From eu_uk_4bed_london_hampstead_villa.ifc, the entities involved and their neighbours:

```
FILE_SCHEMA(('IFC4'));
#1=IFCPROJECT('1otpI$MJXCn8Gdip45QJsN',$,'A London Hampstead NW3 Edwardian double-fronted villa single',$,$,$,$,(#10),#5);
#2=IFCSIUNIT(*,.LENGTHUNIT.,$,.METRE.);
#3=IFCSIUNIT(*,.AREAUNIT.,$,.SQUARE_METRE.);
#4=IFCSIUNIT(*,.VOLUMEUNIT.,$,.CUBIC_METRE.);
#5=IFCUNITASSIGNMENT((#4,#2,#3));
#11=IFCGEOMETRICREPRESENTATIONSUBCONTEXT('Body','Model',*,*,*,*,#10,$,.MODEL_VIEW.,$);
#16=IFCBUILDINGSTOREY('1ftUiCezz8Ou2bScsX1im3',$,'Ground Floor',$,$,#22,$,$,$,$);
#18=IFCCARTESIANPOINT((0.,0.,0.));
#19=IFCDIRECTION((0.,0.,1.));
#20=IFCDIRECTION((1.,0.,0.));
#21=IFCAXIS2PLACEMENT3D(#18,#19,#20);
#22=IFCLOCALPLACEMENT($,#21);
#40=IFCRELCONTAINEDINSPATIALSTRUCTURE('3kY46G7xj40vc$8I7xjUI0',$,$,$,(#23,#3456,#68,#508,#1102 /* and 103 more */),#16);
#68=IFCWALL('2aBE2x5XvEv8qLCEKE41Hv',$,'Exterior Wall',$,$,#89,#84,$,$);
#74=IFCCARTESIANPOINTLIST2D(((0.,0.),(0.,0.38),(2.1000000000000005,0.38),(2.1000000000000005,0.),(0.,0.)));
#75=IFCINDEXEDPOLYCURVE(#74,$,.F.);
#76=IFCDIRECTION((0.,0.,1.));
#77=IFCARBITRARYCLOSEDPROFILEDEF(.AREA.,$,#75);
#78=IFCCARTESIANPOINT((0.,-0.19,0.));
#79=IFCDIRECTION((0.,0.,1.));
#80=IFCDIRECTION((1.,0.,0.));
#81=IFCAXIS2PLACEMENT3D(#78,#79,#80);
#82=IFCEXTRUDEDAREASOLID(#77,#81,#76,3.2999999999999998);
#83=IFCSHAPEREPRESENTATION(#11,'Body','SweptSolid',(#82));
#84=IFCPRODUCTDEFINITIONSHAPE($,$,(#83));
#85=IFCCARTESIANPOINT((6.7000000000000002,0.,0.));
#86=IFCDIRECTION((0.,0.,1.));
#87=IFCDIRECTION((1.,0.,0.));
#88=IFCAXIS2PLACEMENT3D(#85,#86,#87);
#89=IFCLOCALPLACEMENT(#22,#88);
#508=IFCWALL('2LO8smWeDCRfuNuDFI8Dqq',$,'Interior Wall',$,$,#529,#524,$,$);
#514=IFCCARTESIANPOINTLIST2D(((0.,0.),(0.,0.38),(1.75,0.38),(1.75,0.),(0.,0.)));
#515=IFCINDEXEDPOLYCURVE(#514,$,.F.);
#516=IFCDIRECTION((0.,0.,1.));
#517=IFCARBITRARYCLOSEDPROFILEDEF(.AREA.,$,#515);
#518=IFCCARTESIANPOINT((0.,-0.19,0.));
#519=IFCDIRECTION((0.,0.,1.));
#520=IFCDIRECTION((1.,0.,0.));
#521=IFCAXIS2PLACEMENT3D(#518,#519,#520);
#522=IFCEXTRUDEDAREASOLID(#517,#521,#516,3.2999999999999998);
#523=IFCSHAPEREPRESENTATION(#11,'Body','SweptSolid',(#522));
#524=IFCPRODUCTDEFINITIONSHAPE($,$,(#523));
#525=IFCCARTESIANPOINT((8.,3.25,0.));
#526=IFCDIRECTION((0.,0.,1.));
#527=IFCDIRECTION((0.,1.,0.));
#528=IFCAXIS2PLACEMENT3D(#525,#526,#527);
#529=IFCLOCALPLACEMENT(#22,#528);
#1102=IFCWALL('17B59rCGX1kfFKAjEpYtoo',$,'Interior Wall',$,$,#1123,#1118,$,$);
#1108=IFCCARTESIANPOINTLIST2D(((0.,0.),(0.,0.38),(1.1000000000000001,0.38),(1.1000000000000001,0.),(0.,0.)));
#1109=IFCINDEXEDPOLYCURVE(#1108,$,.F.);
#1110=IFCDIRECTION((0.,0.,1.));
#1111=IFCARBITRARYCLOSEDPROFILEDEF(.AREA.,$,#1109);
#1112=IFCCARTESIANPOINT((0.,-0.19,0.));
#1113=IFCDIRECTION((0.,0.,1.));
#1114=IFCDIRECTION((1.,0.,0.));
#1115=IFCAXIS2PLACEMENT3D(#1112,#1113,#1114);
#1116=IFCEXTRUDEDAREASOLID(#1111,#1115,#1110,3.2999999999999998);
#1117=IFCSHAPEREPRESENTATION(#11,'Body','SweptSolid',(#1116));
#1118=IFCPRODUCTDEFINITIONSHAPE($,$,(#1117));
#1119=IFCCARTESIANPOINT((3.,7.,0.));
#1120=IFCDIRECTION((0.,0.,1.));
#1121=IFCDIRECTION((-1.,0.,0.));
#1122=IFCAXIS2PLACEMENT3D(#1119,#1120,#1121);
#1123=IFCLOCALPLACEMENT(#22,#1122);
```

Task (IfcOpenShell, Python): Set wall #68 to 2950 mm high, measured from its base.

```python
import ifcopenshell
import ifcopenshell.geom
import ifcopenshell.util.representation
import ifcopenshell.util.shape
import ifcopenshell.util.unit

model = ifcopenshell.open("eu_uk_4bed_london_hampstead_villa.ifc")
unit_scale = ifcopenshell.util.unit.calculate_unit_scale(model)
settings = ifcopenshell.geom.settings()


def volume(element):
    """Net volume in cubic metres, openings subtracted."""
    shape = ifcopenshell.geom.create_shape(settings, element)
    return ifcopenshell.util.shape.get_volume(shape.geometry)


wall = model.by_guid("2aBE2x5XvEv8qLCEKE41Hv")
before = volume(wall)

body = ifcopenshell.util.representation.get_representation(wall, "Model", "Body")
solid = body.Items[0]
old_height = solid.Depth
solid.Depth = 2.95 / unit_scale
after = volume(wall)

print(f"height {old_height:g} -> {solid.Depth:g}, volume {before:.3f} -> {after:.3f} m3")

model.write("eu_uk_4bed_london_hampstead_villa_updated.ifc")
```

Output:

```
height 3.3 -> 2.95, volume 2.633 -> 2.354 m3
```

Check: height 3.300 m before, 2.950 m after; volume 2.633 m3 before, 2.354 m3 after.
